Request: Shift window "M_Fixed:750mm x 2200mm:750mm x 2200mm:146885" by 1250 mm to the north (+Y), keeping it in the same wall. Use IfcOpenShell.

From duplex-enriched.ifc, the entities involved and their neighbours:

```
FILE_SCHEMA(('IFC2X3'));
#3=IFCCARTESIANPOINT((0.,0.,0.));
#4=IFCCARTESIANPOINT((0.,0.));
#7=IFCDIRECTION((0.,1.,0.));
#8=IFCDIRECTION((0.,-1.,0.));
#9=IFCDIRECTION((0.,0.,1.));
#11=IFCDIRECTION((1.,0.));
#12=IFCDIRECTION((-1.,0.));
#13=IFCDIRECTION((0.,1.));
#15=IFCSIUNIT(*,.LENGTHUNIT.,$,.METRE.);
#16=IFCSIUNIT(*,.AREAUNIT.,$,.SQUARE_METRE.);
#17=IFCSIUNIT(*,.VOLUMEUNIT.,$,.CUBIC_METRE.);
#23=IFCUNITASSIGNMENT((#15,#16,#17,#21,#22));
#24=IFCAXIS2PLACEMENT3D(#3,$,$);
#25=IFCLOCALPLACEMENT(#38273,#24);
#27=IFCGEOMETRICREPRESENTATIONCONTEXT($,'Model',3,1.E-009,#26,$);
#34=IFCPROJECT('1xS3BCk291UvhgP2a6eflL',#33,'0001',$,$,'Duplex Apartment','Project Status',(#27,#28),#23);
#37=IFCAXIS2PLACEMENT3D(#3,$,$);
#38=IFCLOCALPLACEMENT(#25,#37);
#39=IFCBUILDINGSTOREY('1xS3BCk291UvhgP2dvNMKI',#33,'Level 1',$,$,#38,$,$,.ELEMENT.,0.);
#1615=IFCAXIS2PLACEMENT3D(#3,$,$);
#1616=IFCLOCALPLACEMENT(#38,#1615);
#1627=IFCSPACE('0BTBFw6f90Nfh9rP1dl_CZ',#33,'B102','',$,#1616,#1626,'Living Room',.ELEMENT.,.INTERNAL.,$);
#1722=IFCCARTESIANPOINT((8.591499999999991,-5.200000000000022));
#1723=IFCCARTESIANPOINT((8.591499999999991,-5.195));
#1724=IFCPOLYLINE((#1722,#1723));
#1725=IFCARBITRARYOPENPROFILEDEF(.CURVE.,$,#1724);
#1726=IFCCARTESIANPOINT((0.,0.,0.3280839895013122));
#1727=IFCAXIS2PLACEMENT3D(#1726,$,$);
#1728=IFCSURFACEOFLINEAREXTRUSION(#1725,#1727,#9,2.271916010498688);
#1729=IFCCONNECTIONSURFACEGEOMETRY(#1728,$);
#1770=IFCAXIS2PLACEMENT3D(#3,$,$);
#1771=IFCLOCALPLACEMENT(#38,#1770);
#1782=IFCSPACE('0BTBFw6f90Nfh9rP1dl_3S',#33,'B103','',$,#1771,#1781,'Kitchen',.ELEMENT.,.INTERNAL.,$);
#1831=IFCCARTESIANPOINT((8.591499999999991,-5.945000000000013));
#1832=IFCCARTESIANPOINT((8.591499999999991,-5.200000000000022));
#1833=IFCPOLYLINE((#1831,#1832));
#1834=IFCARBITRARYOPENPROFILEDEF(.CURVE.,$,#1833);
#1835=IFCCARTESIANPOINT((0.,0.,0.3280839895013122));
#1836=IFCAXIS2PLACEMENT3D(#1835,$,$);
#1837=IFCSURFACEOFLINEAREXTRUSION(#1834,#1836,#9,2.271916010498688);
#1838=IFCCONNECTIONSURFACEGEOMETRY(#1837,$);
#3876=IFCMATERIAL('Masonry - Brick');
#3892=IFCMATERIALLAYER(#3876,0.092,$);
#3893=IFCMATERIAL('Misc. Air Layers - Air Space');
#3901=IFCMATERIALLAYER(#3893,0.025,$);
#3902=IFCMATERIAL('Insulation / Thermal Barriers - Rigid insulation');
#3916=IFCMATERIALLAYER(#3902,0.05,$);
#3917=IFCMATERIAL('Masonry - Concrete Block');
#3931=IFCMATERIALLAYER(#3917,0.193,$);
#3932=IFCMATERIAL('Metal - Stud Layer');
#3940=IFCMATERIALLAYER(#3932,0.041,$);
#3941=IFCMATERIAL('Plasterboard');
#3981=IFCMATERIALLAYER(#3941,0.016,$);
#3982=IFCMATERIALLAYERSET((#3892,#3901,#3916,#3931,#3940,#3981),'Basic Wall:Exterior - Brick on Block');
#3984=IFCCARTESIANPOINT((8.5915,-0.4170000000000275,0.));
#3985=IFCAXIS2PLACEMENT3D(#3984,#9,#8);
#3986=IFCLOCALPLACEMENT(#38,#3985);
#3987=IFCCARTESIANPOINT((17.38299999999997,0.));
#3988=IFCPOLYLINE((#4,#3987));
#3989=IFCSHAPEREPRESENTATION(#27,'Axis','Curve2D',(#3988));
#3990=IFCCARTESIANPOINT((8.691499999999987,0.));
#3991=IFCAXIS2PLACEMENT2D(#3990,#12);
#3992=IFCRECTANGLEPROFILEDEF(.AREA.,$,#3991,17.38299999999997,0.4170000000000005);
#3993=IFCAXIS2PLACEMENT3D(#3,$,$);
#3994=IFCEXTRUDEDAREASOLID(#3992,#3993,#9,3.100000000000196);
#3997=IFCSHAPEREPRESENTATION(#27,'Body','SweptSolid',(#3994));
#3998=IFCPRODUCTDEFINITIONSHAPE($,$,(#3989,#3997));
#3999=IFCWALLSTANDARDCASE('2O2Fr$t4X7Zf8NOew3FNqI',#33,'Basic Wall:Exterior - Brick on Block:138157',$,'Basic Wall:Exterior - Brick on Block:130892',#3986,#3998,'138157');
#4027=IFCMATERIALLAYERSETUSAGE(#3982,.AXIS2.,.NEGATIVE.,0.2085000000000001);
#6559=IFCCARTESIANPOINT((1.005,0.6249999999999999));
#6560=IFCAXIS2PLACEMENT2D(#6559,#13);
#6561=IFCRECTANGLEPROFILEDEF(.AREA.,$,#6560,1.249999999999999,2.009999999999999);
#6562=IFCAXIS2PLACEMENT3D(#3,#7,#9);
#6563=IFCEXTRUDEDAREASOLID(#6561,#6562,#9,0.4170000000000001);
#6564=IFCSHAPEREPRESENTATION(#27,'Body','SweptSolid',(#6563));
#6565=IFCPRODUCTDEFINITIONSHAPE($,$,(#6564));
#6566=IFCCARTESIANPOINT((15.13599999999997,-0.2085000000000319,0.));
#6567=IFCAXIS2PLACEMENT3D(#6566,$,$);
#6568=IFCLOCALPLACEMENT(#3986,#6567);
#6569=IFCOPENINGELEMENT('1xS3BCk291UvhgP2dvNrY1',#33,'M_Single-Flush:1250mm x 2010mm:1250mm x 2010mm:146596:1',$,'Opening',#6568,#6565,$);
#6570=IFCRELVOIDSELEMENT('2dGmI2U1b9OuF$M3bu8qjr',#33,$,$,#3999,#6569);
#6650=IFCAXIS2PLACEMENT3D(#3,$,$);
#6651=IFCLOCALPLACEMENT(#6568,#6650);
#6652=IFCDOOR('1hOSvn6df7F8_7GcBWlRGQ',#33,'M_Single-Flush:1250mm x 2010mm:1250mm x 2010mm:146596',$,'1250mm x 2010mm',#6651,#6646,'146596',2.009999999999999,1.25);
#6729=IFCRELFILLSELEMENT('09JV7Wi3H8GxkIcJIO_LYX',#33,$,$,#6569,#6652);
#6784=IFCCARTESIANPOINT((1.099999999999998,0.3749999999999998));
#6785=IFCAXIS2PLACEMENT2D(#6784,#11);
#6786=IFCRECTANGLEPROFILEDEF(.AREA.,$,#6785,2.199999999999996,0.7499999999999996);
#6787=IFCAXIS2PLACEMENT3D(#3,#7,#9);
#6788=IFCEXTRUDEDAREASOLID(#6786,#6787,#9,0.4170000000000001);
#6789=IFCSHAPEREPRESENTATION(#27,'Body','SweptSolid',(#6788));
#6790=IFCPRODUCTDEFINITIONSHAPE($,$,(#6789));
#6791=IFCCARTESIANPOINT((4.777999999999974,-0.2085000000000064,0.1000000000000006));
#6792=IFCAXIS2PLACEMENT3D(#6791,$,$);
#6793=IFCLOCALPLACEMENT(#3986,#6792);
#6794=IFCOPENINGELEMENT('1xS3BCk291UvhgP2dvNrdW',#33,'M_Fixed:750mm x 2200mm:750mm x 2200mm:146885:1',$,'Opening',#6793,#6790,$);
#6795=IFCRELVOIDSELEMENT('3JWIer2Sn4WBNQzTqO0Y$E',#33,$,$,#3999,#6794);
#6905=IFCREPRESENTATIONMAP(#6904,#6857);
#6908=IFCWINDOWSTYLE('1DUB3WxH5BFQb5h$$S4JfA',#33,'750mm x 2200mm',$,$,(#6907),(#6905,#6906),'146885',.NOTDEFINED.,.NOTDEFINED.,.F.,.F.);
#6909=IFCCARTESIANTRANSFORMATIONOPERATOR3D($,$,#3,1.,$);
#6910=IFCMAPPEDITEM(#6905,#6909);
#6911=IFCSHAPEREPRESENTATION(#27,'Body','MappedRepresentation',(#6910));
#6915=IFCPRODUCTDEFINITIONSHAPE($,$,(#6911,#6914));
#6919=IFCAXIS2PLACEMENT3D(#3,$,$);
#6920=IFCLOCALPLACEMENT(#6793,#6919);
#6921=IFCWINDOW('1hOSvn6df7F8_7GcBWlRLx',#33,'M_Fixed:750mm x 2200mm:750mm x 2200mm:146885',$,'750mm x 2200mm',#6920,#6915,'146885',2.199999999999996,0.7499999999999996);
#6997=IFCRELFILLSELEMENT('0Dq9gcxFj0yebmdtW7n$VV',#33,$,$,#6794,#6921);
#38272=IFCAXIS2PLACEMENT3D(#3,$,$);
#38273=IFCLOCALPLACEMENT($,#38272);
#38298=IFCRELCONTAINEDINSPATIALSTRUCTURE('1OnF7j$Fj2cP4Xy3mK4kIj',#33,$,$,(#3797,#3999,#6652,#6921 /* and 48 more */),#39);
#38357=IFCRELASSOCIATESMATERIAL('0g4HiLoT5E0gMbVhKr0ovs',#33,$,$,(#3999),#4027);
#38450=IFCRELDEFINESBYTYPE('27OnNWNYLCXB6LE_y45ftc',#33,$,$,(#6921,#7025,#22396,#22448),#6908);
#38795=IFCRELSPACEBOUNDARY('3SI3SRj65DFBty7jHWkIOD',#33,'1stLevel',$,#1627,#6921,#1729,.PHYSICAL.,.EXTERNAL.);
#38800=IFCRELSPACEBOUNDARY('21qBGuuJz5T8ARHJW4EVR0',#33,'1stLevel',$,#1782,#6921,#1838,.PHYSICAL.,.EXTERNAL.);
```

```python
import numpy as np
import ifcopenshell
import ifcopenshell.api.geometry
import ifcopenshell.util.placement
import ifcopenshell.util.unit

model = ifcopenshell.open("duplex-enriched.ifc")
unit_scale = ifcopenshell.util.unit.calculate_unit_scale(model)

window = model.by_id(6921)
opening = window.FillsVoids[0].RelatingOpeningElement
wall = opening.VoidsElements[0].RelatingBuildingElement

wall_matrix = ifcopenshell.util.placement.get_local_placement(wall.ObjectPlacement)
shift = wall_matrix[:3, 0] * -1.25 / unit_scale
before = ifcopenshell.util.placement.get_local_placement(window.ObjectPlacement)[:3, 3].copy()

# The window is placed relative to its opening, so it follows when the opening moves.
matrix = ifcopenshell.util.placement.get_local_placement(opening.ObjectPlacement)
matrix[:3, 3] += shift
ifcopenshell.api.geometry.edit_object_placement(
    model, product=opening, matrix=matrix, is_si=False, should_transform_children=True
)

# Space boundary surfaces are stored in each space's coordinates; move them too.
for rel in window.ProvidesBoundaries:
    if not rel.ConnectionGeometry:
        continue
    surface = rel.ConnectionGeometry.SurfaceOnRelatingElement
    space_matrix = ifcopenshell.util.placement.get_local_placement(rel.RelatingSpace.ObjectPlacement)
    point = np.array(surface.Position.Location.Coordinates) + space_matrix[:3, :3].T @ shift
    surface.Position = model.createIfcAxis2Placement3D(
        model.createIfcCartesianPoint(point.tolist()), surface.Position.Axis, surface.Position.RefDirection
    )

after = ifcopenshell.util.placement.get_local_placement(window.ObjectPlacement)[:3, 3]
print("window moved by", (after - before).round(3) + 0.0)

model.write("duplex-enriched_updated.ifc")
```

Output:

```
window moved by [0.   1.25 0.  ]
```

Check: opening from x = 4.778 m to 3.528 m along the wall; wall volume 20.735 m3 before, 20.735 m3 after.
